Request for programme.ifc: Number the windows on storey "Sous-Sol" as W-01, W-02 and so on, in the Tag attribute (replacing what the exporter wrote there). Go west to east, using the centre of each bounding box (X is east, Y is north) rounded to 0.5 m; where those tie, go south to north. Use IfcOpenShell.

First a look at what the model holds.

```python
import ifcopenshell
import ifcopenshell.util.element
import ifcopenshell.util.placement

model = ifcopenshell.open("programme.ifc")
print(model.schema)
storey = next(s for s in model.by_type("IfcBuildingStorey") if s.Name == "Sous-Sol")
windows = [e for e in ifcopenshell.util.element.get_decomposition(storey) if e.is_a("IfcWindow")]
for e in sorted(windows, key=lambda e: e.id()):
    origin = ifcopenshell.util.placement.get_local_placement(e.ObjectPlacement)[:3, 3]
    print(e.id(), e.Tag, e.Name, origin.round(2) + 0.0, sep=" | ")
```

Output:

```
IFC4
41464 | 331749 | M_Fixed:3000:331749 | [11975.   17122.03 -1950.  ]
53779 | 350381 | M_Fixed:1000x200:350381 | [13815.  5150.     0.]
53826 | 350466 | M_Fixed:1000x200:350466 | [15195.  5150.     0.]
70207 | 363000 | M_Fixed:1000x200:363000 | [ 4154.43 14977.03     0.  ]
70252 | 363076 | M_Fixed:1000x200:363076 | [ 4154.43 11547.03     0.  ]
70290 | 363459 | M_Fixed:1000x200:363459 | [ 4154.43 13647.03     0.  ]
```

```python
import ifcopenshell
import ifcopenshell.geom
import ifcopenshell.util.element
import ifcopenshell.util.shape

model = ifcopenshell.open("programme.ifc")
settings = ifcopenshell.geom.settings()
settings.set("use-world-coords", True)


def centre(element):
    shape = ifcopenshell.geom.create_shape(settings, element)
    return ifcopenshell.util.shape.get_bbox_centroid(shape.geometry)


storey = next(s for s in model.by_type("IfcBuildingStorey") if s.Name == "Sous-Sol")
windows = [e for e in ifcopenshell.util.element.get_decomposition(storey) if e.is_a("IfcWindow")]

# Insertion points can sit at a corner or the storey origin, so sort by the geometry (in metres).
centres = {e: centre(e) for e in windows}
windows.sort(key=lambda e: (round(centres[e][0] / 0.5), centres[e][1]))

for i, e in enumerate(windows, start=1):
    number = f"W-{i:02d}"
    e.Tag = number
    print(e.id(), number)

model.write("programme_rev.ifc")
```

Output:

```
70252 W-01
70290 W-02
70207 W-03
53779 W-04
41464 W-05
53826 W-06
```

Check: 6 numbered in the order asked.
